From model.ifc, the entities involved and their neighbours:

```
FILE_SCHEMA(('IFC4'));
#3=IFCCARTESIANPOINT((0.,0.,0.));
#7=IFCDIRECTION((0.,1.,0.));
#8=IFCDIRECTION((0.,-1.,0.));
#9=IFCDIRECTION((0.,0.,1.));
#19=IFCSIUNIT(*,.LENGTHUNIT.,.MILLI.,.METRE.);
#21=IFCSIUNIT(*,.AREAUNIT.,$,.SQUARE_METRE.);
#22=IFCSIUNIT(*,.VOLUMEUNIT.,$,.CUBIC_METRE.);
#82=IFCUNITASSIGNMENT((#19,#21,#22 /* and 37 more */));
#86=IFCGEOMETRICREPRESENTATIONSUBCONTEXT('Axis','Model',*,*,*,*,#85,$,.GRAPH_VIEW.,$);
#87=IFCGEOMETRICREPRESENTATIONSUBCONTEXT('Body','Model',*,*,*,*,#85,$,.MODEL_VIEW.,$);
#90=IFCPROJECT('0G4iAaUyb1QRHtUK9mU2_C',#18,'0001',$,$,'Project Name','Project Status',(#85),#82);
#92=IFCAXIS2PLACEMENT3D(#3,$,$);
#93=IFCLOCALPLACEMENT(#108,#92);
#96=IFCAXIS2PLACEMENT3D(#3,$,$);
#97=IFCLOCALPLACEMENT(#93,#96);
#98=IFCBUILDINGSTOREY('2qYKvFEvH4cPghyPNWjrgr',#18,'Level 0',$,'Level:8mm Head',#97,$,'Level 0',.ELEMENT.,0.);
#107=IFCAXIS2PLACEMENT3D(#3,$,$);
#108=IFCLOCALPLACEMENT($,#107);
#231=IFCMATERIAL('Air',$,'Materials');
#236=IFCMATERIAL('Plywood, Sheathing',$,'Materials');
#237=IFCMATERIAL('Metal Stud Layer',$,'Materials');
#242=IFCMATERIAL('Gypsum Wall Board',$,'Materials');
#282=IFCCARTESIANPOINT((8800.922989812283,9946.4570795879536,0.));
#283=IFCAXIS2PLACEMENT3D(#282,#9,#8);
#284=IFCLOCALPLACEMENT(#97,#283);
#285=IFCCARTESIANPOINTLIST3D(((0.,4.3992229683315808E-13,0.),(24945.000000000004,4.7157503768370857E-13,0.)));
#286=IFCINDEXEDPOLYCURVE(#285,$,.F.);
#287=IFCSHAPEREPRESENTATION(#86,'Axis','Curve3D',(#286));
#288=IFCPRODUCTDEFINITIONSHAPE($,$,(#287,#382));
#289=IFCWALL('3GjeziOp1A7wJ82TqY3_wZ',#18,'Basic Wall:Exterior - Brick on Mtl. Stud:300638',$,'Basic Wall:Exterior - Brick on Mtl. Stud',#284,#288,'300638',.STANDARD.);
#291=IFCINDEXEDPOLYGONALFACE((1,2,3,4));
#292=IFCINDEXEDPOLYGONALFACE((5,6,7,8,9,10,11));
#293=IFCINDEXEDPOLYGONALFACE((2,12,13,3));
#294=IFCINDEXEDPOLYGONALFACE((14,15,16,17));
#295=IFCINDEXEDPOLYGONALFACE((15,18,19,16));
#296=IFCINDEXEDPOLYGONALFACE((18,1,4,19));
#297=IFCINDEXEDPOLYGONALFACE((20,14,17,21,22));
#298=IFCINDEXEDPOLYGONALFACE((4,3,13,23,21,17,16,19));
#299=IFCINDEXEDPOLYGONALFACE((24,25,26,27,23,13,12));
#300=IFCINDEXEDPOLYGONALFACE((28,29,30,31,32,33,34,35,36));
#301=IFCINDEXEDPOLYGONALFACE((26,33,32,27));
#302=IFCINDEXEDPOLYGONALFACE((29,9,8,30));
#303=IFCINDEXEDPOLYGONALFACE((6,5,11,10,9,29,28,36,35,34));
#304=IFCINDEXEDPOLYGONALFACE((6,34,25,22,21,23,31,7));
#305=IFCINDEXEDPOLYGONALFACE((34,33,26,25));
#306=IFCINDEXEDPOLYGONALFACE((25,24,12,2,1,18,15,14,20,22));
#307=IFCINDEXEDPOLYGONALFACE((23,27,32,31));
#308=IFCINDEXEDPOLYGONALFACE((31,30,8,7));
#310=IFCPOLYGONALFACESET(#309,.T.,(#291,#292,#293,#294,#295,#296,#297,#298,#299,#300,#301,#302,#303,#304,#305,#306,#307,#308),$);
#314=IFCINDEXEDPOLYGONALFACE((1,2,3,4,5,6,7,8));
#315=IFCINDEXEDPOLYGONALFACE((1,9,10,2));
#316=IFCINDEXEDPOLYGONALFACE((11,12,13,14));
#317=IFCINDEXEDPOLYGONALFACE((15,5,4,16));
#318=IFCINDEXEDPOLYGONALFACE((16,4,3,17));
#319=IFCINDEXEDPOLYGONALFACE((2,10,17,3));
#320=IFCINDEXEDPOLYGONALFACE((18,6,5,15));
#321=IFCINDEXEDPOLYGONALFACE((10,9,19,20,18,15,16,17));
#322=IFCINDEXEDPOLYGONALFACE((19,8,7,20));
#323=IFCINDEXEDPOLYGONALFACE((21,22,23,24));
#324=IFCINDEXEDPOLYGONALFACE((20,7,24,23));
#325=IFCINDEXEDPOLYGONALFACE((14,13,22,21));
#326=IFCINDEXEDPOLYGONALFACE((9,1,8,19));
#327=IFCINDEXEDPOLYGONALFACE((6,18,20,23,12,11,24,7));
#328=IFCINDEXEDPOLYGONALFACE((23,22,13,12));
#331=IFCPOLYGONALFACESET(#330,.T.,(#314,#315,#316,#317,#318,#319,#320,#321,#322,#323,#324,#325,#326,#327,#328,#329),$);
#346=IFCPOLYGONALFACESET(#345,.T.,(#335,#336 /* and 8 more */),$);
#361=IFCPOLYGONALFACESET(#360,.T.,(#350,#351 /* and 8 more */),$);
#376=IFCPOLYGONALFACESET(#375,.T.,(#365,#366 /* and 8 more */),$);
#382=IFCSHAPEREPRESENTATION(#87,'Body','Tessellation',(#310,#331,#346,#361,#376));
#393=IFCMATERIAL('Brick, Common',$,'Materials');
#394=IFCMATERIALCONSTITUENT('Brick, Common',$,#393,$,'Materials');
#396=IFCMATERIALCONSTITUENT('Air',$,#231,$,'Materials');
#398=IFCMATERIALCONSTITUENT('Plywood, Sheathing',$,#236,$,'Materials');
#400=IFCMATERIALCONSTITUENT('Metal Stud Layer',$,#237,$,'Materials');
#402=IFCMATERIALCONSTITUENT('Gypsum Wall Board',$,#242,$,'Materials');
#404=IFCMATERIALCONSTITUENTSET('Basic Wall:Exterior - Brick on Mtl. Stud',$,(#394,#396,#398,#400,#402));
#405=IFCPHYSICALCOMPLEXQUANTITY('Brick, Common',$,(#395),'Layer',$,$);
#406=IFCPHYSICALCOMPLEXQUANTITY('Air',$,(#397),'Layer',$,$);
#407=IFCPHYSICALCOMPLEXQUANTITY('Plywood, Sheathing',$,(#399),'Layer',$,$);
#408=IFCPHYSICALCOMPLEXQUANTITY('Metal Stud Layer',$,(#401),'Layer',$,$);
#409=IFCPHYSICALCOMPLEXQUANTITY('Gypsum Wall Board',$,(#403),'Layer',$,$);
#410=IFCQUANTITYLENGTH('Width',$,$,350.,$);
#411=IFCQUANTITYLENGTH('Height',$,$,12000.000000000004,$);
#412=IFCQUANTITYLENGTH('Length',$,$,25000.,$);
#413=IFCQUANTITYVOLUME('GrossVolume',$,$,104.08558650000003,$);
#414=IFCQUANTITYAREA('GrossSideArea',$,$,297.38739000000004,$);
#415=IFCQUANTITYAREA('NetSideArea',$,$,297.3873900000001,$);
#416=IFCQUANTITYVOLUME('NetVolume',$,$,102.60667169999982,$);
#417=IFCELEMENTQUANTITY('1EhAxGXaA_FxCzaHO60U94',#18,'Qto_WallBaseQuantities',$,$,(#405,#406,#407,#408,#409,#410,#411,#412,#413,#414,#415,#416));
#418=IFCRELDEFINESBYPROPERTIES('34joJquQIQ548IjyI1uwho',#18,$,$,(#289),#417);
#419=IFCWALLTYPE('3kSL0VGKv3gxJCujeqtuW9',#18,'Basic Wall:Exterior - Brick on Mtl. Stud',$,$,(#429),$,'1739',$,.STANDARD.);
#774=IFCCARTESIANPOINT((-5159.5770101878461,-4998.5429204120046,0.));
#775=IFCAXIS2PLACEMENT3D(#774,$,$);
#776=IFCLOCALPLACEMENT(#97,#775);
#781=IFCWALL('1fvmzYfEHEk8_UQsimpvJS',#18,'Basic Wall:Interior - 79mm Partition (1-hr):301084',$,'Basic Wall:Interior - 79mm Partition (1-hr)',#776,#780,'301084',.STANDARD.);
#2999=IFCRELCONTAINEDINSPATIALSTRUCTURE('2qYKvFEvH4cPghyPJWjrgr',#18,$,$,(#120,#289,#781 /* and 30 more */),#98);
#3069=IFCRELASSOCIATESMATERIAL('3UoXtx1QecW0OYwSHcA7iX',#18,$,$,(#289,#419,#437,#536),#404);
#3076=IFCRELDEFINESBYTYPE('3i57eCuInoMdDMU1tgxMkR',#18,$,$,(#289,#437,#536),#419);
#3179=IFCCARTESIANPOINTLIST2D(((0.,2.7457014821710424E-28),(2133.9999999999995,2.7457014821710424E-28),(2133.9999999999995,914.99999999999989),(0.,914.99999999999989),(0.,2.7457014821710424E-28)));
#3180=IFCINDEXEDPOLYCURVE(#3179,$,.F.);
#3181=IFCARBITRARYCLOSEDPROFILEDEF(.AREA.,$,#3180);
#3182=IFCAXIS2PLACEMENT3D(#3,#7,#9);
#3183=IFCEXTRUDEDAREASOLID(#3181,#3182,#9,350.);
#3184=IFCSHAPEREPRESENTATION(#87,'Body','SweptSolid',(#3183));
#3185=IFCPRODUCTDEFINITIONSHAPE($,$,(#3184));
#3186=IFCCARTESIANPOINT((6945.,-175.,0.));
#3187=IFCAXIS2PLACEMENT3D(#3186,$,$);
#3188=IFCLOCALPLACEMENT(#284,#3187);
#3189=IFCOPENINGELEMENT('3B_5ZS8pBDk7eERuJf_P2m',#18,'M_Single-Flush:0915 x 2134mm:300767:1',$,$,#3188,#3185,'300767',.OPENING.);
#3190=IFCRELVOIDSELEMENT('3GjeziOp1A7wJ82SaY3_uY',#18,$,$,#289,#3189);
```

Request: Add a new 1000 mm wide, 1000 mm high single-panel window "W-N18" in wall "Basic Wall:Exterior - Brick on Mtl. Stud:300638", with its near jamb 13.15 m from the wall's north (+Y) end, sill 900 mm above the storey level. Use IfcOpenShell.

```python
import numpy as np
import ifcopenshell
import ifcopenshell.api.feature
import ifcopenshell.api.geometry
import ifcopenshell.api.pset
import ifcopenshell.api.root
import ifcopenshell.api.spatial
import ifcopenshell.geom
import ifcopenshell.util.element
import ifcopenshell.util.placement
import ifcopenshell.util.representation
import ifcopenshell.util.shape
import ifcopenshell.util.unit

model = ifcopenshell.open("model.ifc")
unit_scale = ifcopenshell.util.unit.calculate_unit_scale(model)
area_scale = ifcopenshell.util.unit.calculate_unit_scale(model, "AREAUNIT")
volume_scale = ifcopenshell.util.unit.calculate_unit_scale(model, "VOLUMEUNIT")
settings = ifcopenshell.geom.settings()


def volume(element):
    """Net volume in cubic metres, openings subtracted."""
    shape = ifcopenshell.geom.create_shape(settings, element)
    return ifcopenshell.util.shape.get_volume(shape.geometry)


wall = model.by_id(289)
storey = ifcopenshell.util.element.get_container(wall, ifc_class="IfcBuildingStorey")
context = ifcopenshell.util.representation.get_context(model, "Model", "Body", "MODEL_VIEW")
before = volume(wall)

width, height, from_end, sill = 1, 1, 13.15, 0.9  # metres

# The wall runs along its own X axis, and the end named is its -X end.
wall_shape = ifcopenshell.geom.create_shape(settings, wall)
x, y, z = ifcopenshell.util.shape.get_vertices(wall_shape.geometry).T
start = x.min() + from_end
face, thickness = float(y.min()), float(y.max() - y.min())
wall_matrix = ifcopenshell.util.placement.get_local_placement(wall.ObjectPlacement)
level = ifcopenshell.util.placement.get_local_placement(storey.ObjectPlacement)[2, 3]


def in_wall(x, y):
    """Placement at x, y metres in the wall's axes, at sill height."""
    matrix = wall_matrix.copy()
    matrix[:, 3] = wall_matrix @ np.array([x / unit_scale, y / unit_scale, 0.0, 1.0])
    matrix[2, 3] = level + sill / unit_scale
    return matrix


# Opening: a box that overshoots both wall faces by 50 mm.
opening = ifcopenshell.api.root.create_entity(model, ifc_class="IfcOpeningElement", predefined_type="OPENING")
box = ifcopenshell.api.geometry.add_wall_representation(
    model, context=context, length=width, height=height, thickness=thickness + 0.1
)
ifcopenshell.api.geometry.assign_representation(model, product=opening, representation=box)
ifcopenshell.api.geometry.edit_object_placement(model, product=opening, matrix=in_wall(start, face - 0.05), is_si=False)
ifcopenshell.api.feature.add_feature(model, feature=opening, element=wall)

window = ifcopenshell.api.root.create_entity(model, ifc_class="IfcWindow", name="W-N18", predefined_type="WINDOW")
window.OverallWidth, window.OverallHeight = width / unit_scale, height / unit_scale
window.PartitioningType = "SINGLE_PANEL"
body = ifcopenshell.api.geometry.add_window_representation(
    model,
    context=context,
    overall_width=window.OverallWidth,
    overall_height=window.OverallHeight,
    partition_type="SINGLE_PANEL",
)
ifcopenshell.api.geometry.assign_representation(model, product=window, representation=body)
ifcopenshell.api.spatial.assign_container(model, products=[window], relating_structure=storey)
ifcopenshell.api.feature.add_filling(model, opening=opening, element=window)

# Centre the window in the wall's thickness.
ifcopenshell.api.geometry.edit_object_placement(model, product=window, matrix=in_wall(start, face), is_si=False)
window_shape = ifcopenshell.geom.create_shape(settings, window)
depth = ifcopenshell.util.shape.get_vertices(window_shape.geometry)[:, 1]
offset = face + thickness / 2 - (depth.min() + depth.max()) / 2
ifcopenshell.api.geometry.edit_object_placement(model, product=window, matrix=in_wall(start, offset), is_si=False)

after = volume(wall)

# Update the wall's stored quantities.
qto = model.by_id(ifcopenshell.util.element.get_pset(wall, "Qto_WallBaseQuantities", should_inherit=False)["id"])
ifcopenshell.api.pset.edit_qto(model, qto=qto, properties={
    "NetSideArea": after / thickness / area_scale,
    "NetVolume": after / volume_scale,
})

print(f"wall volume {before:.3f} -> {after:.3f} m3")

model.write("model_edited.ifc")
```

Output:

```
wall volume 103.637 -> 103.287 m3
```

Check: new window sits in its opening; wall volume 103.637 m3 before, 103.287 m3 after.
